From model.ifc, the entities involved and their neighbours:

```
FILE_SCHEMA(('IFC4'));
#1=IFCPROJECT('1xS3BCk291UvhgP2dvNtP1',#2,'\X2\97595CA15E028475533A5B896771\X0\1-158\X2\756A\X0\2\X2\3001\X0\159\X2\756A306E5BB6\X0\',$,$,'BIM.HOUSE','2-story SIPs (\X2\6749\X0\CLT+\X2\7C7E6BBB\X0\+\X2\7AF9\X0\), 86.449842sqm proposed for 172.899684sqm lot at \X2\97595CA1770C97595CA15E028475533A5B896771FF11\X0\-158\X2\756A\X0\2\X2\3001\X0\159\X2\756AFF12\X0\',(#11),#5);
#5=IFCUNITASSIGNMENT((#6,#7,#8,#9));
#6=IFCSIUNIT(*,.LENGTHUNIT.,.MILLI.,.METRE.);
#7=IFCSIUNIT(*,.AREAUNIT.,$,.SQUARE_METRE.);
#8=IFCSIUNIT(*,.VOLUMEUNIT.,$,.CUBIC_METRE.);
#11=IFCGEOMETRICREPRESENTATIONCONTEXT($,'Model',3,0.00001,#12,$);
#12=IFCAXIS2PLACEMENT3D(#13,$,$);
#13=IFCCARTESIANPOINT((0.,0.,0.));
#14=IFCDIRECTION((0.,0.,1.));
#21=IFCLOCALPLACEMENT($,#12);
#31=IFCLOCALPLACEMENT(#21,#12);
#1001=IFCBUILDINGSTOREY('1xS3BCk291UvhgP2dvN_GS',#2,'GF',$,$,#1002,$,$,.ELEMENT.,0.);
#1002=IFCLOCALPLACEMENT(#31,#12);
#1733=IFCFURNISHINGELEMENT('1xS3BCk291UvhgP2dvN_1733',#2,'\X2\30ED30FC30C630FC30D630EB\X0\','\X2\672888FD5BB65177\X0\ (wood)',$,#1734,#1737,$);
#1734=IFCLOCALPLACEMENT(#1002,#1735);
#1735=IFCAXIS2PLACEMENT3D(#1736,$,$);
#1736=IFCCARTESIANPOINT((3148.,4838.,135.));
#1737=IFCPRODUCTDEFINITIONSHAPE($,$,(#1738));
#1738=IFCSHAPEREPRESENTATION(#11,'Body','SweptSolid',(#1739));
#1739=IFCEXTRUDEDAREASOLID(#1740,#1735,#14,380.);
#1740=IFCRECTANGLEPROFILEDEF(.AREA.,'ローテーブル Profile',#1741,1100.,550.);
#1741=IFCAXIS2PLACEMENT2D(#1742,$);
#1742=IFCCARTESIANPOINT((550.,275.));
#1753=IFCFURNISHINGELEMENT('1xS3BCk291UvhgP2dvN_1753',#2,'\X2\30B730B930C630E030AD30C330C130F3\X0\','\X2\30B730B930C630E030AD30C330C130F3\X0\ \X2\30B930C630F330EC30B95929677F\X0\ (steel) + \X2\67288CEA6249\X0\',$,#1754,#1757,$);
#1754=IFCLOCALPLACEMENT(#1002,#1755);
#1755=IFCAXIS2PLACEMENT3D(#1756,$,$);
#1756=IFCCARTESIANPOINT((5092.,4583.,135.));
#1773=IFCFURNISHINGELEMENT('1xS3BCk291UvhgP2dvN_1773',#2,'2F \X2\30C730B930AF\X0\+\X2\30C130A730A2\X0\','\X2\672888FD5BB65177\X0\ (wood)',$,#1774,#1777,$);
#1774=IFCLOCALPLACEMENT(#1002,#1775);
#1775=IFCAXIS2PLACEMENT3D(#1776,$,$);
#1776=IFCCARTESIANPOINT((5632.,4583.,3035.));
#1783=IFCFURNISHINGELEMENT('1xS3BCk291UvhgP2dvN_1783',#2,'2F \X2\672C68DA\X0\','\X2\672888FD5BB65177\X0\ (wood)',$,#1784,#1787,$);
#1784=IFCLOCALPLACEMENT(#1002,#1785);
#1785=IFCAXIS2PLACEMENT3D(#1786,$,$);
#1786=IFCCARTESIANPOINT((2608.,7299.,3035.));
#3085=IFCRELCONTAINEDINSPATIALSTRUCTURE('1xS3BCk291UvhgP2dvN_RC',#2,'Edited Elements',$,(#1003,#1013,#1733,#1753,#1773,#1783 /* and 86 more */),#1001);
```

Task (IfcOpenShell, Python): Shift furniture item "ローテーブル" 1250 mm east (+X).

```python
import ifcopenshell
import ifcopenshell.api.geometry
import ifcopenshell.util.placement
import ifcopenshell.util.unit

model = ifcopenshell.open("model.ifc")
unit_scale = ifcopenshell.util.unit.calculate_unit_scale(model)

item = model.by_id(1733)
matrix = ifcopenshell.util.placement.get_local_placement(item.ObjectPlacement)
matrix[0, 3] += 1.25 / unit_scale
ifcopenshell.api.geometry.edit_object_placement(model, product=item, matrix=matrix, is_si=False)

print(ifcopenshell.util.placement.get_local_placement(item.ObjectPlacement).round(3) + 0.0)

model.write("model_updated.ifc")
```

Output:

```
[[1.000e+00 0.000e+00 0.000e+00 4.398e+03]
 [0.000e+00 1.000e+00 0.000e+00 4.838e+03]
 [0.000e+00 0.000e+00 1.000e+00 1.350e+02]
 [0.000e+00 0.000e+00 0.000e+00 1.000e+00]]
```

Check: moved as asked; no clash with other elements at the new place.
